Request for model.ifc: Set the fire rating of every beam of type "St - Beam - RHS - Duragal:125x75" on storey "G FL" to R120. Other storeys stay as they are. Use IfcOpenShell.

First a look at what the model holds.

```python
import ifcopenshell
import ifcopenshell.util.element

model = ifcopenshell.open("model.ifc")
print(model.schema)
storey = next(s for s in model.by_type("IfcBuildingStorey") if s.Name == "G FL")
beams = [e for e in ifcopenshell.util.element.get_decomposition(storey) if e.is_a("IfcBeam")]
seen = {}
for e in beams:
    element_type = ifcopenshell.util.element.get_type(e)
    key = (element_type.Name if element_type != e and element_type else None, ifcopenshell.util.element.get_pset(e, "Pset_BeamCommon", "FireRating"))
    seen[key] = seen.get(key, 0) + 1
for (name, value), count in sorted(seen.items(), key=str):
    print(count, "x", name, "|", value)
```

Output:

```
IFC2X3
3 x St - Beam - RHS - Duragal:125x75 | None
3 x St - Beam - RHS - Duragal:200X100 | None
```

```python
import ifcopenshell
import ifcopenshell.api.pset
import ifcopenshell.util.element

model = ifcopenshell.open("model.ifc")

storey = next(s for s in model.by_type("IfcBuildingStorey") if s.Name == "G FL")
beams = [e for e in ifcopenshell.util.element.get_decomposition(storey) if e.is_a("IfcBeam")]

count = 0
for e in beams:
    element_type = ifcopenshell.util.element.get_type(e)
    if element_type in (None, e) or element_type.Name != "St - Beam - RHS - Duragal:125x75":
        continue
    # add_pset returns the element's existing set when there is one.
    pset = ifcopenshell.api.pset.add_pset(model, product=e, name="Pset_BeamCommon")
    ifcopenshell.api.pset.edit_pset(model, pset=pset, properties={"FireRating": "R120"})
    count += 1

print(count, "beams updated")

model.write("model_edited.ifc")
```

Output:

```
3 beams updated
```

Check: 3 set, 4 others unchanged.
